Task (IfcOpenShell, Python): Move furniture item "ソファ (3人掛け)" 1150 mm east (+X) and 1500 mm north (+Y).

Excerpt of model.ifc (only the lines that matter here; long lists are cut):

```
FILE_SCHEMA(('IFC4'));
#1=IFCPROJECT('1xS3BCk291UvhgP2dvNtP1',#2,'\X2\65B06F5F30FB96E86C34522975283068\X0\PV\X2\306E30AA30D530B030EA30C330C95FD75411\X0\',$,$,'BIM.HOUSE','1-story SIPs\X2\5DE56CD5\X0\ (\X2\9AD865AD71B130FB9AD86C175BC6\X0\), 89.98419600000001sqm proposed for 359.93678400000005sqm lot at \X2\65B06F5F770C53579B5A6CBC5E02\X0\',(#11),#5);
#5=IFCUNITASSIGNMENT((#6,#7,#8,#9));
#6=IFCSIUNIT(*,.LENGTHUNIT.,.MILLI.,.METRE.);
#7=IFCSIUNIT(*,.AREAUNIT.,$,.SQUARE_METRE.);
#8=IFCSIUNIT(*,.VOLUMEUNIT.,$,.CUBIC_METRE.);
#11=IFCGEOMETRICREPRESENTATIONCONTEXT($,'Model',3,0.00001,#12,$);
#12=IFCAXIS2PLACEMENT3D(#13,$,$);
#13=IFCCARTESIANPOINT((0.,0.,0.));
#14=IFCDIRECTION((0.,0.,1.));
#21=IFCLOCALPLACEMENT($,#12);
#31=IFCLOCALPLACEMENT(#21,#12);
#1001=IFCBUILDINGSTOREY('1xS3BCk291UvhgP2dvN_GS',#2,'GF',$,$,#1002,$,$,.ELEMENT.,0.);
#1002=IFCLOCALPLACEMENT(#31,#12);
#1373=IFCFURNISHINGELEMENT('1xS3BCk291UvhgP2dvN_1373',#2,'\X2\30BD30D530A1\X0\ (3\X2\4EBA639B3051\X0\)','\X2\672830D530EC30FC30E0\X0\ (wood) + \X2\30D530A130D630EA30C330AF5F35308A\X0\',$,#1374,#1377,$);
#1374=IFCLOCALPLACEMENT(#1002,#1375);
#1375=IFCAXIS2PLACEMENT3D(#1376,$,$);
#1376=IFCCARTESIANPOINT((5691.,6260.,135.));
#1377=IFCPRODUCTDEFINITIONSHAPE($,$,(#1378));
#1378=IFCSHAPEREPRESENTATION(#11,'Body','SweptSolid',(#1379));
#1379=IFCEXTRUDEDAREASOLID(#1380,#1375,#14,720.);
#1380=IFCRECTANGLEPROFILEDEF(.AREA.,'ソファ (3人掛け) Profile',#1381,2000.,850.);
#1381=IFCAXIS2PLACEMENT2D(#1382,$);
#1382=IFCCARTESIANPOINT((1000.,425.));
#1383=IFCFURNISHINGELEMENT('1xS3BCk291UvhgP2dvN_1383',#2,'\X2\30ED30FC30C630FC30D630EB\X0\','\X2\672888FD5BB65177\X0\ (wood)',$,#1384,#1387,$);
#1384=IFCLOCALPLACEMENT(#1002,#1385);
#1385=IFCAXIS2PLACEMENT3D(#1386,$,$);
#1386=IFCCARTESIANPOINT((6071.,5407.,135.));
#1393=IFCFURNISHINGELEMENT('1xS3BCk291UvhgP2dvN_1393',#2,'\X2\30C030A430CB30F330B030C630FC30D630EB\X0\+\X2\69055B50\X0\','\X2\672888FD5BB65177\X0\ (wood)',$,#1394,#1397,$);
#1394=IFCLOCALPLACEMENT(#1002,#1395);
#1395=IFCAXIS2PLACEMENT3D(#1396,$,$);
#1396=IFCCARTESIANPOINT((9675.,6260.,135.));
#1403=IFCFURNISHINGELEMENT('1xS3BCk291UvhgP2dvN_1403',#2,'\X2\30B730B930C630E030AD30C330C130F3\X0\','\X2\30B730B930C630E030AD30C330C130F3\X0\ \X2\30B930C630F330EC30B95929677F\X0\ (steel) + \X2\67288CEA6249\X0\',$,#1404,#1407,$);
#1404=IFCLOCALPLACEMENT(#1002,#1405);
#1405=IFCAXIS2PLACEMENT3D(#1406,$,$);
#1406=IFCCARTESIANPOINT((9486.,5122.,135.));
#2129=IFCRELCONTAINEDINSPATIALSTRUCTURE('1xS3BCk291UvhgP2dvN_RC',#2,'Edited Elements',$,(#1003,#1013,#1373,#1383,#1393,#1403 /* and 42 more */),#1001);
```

```python
import ifcopenshell
import ifcopenshell.api.geometry
import ifcopenshell.util.placement
import ifcopenshell.util.unit

model = ifcopenshell.open("model.ifc")
unit_scale = ifcopenshell.util.unit.calculate_unit_scale(model)

item = model.by_guid("1xS3BCk291UvhgP2dvN_1373")
matrix = ifcopenshell.util.placement.get_local_placement(item.ObjectPlacement)
matrix[0, 3] += 1.15 / unit_scale
matrix[1, 3] += 1.5 / unit_scale
ifcopenshell.api.geometry.edit_object_placement(model, product=item, matrix=matrix, is_si=False)

print(ifcopenshell.util.placement.get_local_placement(item.ObjectPlacement).round(3) + 0.0)

model.write("model_rev.ifc")
```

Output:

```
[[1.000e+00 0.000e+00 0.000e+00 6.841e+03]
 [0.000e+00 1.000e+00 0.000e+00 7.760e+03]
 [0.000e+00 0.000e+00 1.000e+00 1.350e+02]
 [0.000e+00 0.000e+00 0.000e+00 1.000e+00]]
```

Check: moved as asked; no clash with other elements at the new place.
